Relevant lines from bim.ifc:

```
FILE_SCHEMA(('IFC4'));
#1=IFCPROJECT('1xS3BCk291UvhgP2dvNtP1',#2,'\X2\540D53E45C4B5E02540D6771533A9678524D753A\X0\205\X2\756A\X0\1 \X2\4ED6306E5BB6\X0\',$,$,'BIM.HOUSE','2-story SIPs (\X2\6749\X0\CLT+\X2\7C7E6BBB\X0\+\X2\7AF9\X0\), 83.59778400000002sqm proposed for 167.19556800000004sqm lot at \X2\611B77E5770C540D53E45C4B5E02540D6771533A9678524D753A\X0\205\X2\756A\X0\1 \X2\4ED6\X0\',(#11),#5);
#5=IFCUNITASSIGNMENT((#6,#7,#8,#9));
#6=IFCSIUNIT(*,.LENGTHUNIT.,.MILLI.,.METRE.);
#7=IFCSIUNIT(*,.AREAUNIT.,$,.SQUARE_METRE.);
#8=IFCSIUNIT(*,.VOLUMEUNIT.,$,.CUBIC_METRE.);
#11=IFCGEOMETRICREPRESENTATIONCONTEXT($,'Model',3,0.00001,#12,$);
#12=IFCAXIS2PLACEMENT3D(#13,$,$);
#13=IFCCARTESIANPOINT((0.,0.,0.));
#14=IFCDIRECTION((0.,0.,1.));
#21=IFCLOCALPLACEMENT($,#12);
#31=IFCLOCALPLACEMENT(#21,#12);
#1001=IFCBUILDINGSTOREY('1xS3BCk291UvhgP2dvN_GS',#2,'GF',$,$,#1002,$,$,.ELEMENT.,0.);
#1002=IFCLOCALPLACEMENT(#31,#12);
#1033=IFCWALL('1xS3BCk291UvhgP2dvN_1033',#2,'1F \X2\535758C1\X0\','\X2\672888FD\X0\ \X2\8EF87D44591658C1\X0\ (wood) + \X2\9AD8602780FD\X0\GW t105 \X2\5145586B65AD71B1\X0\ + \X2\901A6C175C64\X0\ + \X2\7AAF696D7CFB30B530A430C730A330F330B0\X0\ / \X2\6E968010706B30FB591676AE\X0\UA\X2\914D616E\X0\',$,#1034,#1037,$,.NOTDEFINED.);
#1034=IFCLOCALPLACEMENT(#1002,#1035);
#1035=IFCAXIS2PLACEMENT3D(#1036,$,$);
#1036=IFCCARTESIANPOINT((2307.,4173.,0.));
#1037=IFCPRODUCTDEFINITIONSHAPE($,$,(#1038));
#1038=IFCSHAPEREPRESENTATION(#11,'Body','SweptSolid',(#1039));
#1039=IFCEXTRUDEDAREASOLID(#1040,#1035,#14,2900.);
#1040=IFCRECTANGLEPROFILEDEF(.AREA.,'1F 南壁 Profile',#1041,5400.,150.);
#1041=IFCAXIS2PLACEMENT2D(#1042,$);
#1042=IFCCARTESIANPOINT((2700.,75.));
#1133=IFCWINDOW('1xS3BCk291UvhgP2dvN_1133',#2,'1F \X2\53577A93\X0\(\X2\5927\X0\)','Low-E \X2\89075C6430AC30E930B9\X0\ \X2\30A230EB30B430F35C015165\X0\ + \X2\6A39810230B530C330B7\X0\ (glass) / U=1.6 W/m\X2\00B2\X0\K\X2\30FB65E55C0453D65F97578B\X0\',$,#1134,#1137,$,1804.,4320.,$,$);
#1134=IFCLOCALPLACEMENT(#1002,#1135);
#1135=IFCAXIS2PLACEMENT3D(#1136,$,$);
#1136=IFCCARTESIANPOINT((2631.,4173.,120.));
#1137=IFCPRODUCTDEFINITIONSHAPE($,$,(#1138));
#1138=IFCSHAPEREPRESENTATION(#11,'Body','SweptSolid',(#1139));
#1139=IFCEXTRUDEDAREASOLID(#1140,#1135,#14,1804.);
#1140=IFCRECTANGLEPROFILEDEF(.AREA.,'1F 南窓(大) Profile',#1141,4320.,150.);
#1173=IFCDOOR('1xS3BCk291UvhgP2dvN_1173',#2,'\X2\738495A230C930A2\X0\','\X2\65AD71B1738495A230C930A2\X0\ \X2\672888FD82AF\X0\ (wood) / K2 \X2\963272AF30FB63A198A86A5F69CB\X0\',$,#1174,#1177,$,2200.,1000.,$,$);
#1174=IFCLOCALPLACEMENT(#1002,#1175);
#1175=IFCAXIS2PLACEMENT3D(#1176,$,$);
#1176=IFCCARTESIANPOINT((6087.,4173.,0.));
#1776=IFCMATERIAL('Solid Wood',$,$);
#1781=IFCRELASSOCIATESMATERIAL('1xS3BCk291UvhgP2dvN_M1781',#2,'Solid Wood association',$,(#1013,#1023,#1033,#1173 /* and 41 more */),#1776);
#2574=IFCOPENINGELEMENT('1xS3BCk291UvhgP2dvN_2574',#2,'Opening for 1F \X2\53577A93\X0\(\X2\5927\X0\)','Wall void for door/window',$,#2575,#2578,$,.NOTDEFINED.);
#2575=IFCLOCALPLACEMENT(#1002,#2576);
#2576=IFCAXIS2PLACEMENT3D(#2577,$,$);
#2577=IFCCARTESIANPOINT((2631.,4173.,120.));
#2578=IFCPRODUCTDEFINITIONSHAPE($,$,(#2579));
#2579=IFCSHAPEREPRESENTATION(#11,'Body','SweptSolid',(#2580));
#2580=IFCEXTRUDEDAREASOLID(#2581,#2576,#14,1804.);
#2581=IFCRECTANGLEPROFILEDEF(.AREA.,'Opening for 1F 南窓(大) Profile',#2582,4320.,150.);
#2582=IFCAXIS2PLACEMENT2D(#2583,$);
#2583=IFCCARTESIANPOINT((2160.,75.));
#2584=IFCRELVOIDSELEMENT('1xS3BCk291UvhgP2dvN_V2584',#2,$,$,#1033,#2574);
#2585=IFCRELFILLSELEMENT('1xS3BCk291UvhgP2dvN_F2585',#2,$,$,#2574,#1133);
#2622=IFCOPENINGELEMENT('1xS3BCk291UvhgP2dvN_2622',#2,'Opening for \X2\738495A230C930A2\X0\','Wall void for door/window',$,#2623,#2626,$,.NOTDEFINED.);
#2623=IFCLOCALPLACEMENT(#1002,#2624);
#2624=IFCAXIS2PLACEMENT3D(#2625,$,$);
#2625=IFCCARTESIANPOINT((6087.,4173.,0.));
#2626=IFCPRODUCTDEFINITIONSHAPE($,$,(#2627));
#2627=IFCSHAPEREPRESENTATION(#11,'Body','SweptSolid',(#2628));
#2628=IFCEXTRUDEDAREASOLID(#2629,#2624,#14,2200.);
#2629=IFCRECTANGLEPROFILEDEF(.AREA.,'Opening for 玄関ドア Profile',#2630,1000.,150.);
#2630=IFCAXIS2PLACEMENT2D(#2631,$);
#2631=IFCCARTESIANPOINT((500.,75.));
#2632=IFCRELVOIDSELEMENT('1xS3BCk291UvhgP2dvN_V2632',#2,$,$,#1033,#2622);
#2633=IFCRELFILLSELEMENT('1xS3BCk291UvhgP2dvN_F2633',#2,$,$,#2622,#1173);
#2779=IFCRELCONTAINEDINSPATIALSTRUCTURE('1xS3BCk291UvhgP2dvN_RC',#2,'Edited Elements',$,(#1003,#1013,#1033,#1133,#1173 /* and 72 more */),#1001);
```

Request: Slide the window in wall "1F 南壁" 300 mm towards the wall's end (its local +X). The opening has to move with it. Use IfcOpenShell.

```python
import ifcopenshell
import ifcopenshell.api.geometry
import ifcopenshell.util.placement

model = ifcopenshell.open("bim.ifc")

window = model.by_guid("1xS3BCk291UvhgP2dvN_1133")
opening = window.FillsVoids[0].RelatingOpeningElement
wall = opening.VoidsElements[0].RelatingBuildingElement

wall_matrix = ifcopenshell.util.placement.get_local_placement(wall.ObjectPlacement)
shift = wall_matrix[:3, 0] * 300.0
before = ifcopenshell.util.placement.get_local_placement(window.ObjectPlacement)[:3, 3].copy()

# The window is not placed relative to its opening, so move both.
for product in (opening, window):
    matrix = ifcopenshell.util.placement.get_local_placement(product.ObjectPlacement)
    matrix[:3, 3] += shift
    ifcopenshell.api.geometry.edit_object_placement(model, product=product, matrix=matrix, is_si=False)

after = ifcopenshell.util.placement.get_local_placement(window.ObjectPlacement)[:3, 3]
print("window moved by", (after - before).round(3) + 0.0)

model.write("bim_v2.ifc")
```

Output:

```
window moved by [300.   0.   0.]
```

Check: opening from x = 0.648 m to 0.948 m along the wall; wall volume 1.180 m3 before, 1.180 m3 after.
